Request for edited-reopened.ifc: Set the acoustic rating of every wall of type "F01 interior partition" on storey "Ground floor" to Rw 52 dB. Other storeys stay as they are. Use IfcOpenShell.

First a look at what the model holds.

```python
import ifcopenshell
import ifcopenshell.util.element

model = ifcopenshell.open("edited-reopened.ifc")
print(model.schema)
storey = next(s for s in model.by_type("IfcBuildingStorey") if s.Name == "Ground floor")
walls = [e for e in ifcopenshell.util.element.get_decomposition(storey) if e.is_a("IfcWall")]
seen = {}
for e in walls:
    element_type = ifcopenshell.util.element.get_type(e)
    key = (element_type.Name if element_type != e and element_type else None, ifcopenshell.util.element.get_pset(e, "Pset_WallCommon", "AcousticRating"))
    seen[key] = seen.get(key, 0) + 1
for (name, value), count in sorted(seen.items(), key=str):
    print(count, "x", name, "|", value)
```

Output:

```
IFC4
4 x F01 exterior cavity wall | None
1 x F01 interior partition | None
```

```python
import ifcopenshell
import ifcopenshell.api.pset
import ifcopenshell.util.element

model = ifcopenshell.open("edited-reopened.ifc")

storey = next(s for s in model.by_type("IfcBuildingStorey") if s.Name == "Ground floor")
walls = [e for e in ifcopenshell.util.element.get_decomposition(storey) if e.is_a("IfcWall")]

count = 0
for e in walls:
    element_type = ifcopenshell.util.element.get_type(e)
    if element_type in (None, e) or element_type.Name != "F01 interior partition":
        continue
    # add_pset returns the element's existing set when there is one.
    pset = ifcopenshell.api.pset.add_pset(model, product=e, name="Pset_WallCommon")
    ifcopenshell.api.pset.edit_pset(model, pset=pset, properties={"AcousticRating": "Rw 52 dB"})
    count += 1

print(count, "walls updated")

model.write("edited-reopened_rev.ifc")
```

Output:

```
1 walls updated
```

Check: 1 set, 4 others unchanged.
